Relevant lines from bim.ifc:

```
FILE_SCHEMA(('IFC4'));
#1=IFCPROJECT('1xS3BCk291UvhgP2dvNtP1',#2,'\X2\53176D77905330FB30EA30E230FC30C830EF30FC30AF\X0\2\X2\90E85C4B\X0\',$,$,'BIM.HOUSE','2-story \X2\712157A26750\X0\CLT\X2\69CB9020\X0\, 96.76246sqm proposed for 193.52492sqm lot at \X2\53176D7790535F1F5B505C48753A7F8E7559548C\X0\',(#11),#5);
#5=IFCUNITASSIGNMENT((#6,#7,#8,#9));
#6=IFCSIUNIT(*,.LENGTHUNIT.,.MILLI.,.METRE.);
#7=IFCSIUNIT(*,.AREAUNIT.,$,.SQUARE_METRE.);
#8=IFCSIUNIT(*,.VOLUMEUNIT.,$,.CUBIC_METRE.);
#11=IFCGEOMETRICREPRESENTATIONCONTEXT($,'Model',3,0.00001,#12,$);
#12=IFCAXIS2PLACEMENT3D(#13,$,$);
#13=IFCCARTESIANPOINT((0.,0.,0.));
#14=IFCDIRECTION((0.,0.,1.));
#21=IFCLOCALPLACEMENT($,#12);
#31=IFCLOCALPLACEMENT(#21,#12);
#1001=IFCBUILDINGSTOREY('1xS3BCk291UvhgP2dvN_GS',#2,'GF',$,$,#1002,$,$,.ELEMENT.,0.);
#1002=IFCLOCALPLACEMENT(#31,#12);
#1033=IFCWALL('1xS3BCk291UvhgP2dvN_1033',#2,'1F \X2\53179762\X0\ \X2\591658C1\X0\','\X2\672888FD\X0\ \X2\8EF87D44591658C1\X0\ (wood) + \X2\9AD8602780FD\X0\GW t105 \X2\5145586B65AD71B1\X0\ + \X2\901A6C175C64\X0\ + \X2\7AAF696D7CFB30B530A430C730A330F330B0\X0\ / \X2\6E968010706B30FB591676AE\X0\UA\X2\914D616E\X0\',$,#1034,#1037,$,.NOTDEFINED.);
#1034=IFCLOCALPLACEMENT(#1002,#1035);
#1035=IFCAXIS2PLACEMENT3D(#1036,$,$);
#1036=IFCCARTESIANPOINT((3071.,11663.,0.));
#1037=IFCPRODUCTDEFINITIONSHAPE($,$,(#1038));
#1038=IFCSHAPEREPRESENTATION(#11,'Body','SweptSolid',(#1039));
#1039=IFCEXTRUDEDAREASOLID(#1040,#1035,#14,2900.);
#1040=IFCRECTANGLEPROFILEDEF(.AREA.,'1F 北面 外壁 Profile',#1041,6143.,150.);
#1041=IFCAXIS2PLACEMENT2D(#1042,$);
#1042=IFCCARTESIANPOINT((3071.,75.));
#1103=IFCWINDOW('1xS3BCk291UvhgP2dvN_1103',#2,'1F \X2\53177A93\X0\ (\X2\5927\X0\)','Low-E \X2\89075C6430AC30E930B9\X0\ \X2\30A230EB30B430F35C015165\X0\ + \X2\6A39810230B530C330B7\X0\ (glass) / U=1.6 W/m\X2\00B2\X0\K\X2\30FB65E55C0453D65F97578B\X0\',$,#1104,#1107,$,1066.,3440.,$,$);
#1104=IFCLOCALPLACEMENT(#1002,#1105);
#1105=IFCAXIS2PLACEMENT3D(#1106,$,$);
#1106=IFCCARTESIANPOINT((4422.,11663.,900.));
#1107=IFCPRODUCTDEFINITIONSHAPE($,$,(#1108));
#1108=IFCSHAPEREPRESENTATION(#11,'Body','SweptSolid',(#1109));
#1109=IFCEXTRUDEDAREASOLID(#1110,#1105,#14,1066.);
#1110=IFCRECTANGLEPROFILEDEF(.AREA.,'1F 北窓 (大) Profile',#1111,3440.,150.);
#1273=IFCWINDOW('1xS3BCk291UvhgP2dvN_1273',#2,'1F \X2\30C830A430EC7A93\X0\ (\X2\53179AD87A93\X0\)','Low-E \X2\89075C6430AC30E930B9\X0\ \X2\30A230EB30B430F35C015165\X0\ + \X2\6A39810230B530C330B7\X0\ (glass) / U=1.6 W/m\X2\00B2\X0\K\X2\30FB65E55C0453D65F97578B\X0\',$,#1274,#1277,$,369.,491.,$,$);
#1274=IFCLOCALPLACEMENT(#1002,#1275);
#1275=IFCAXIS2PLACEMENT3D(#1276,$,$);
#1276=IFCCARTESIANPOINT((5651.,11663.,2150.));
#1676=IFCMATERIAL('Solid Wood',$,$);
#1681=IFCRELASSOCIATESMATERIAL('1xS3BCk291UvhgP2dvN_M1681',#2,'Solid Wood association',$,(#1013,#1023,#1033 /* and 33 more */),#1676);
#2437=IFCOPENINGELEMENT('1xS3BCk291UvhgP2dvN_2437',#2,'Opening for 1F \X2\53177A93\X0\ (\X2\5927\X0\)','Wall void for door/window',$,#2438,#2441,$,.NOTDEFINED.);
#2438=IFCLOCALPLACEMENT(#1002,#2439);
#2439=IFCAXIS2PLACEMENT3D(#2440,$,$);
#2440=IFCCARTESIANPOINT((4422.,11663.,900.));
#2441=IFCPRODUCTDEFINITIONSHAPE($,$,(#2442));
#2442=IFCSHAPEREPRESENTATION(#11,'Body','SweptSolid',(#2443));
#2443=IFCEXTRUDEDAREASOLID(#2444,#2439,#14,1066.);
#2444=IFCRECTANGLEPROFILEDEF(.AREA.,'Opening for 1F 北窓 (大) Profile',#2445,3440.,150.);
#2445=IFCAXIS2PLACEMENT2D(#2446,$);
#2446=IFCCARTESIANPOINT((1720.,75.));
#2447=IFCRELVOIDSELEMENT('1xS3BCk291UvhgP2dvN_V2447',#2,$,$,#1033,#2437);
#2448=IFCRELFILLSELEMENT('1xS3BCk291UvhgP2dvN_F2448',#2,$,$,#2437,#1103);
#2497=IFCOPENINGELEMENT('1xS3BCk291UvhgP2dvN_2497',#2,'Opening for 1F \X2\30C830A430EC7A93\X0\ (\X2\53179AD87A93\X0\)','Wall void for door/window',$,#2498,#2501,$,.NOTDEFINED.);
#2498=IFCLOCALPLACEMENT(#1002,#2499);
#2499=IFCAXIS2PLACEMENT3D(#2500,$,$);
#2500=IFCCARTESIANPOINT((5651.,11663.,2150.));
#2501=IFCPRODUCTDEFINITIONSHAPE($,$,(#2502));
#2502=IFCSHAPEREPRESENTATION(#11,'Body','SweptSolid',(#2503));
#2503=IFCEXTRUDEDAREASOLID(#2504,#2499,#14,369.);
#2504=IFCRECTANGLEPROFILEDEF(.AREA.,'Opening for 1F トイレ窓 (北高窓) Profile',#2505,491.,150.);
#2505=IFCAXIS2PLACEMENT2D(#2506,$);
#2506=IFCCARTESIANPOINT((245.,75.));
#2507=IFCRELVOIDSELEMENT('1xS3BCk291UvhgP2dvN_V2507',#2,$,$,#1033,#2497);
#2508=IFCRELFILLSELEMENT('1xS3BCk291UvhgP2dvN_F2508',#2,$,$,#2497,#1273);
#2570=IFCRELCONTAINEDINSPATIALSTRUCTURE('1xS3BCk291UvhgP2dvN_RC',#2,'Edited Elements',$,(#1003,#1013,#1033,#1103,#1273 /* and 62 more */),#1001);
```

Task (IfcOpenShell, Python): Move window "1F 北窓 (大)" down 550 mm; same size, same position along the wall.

```python
import numpy as np
import ifcopenshell
import ifcopenshell.api.geometry
import ifcopenshell.util.placement
import ifcopenshell.util.unit

model = ifcopenshell.open("bim.ifc")
unit_scale = ifcopenshell.util.unit.calculate_unit_scale(model)

window = model.by_guid("1xS3BCk291UvhgP2dvN_1103")
opening = window.FillsVoids[0].RelatingOpeningElement
dz = -0.55 / unit_scale

shift = np.array([0.0, 0.0, dz])
# The window is not placed relative to its opening, so move both.
for product in (opening, window):
    matrix = ifcopenshell.util.placement.get_local_placement(product.ObjectPlacement)
    matrix[:3, 3] += shift
    ifcopenshell.api.geometry.edit_object_placement(model, product=product, matrix=matrix, is_si=False)

print(f"moved by {dz * unit_scale:+.3f} m")

model.write("bim_edited.ifc")
```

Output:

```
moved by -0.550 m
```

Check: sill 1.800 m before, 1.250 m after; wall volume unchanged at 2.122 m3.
